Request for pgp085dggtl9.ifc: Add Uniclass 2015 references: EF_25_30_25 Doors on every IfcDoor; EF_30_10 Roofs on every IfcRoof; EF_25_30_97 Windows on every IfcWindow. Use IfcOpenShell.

First a look at what the model holds.

```python
import ifcopenshell

model = ifcopenshell.open("pgp085dggtl9.ifc")
print(model.schema)
print("classifications:", [c.Name for c in model.by_type("IfcClassification")])
for ifc_class in ("IfcDoor", "IfcRoof", "IfcStair", "IfcWall", "IfcWindow"):
    print(ifc_class, len(model.by_type(ifc_class)))
```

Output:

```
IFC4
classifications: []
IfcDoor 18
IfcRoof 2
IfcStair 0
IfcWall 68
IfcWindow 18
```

```python
import ifcopenshell
import ifcopenshell.api.classification

model = ifcopenshell.open("pgp085dggtl9.ifc")

system = ifcopenshell.api.classification.add_classification(model, classification="Uniclass 2015")

codes = {
    "IfcDoor": ("EF_25_30_25", "Doors"),
    "IfcRoof": ("EF_30_10", "Roofs"),
    "IfcWindow": ("EF_25_30_97", "Windows"),
}
for ifc_class, (code, name) in codes.items():
    products = model.by_type(ifc_class)
    ifcopenshell.api.classification.add_reference(
        model, products=products, classification=system, identification=code, name=name
    )
    print(code, len(products))

model.write("pgp085dggtl9_edited.ifc")
```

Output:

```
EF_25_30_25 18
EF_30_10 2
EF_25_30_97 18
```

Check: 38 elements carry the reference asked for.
